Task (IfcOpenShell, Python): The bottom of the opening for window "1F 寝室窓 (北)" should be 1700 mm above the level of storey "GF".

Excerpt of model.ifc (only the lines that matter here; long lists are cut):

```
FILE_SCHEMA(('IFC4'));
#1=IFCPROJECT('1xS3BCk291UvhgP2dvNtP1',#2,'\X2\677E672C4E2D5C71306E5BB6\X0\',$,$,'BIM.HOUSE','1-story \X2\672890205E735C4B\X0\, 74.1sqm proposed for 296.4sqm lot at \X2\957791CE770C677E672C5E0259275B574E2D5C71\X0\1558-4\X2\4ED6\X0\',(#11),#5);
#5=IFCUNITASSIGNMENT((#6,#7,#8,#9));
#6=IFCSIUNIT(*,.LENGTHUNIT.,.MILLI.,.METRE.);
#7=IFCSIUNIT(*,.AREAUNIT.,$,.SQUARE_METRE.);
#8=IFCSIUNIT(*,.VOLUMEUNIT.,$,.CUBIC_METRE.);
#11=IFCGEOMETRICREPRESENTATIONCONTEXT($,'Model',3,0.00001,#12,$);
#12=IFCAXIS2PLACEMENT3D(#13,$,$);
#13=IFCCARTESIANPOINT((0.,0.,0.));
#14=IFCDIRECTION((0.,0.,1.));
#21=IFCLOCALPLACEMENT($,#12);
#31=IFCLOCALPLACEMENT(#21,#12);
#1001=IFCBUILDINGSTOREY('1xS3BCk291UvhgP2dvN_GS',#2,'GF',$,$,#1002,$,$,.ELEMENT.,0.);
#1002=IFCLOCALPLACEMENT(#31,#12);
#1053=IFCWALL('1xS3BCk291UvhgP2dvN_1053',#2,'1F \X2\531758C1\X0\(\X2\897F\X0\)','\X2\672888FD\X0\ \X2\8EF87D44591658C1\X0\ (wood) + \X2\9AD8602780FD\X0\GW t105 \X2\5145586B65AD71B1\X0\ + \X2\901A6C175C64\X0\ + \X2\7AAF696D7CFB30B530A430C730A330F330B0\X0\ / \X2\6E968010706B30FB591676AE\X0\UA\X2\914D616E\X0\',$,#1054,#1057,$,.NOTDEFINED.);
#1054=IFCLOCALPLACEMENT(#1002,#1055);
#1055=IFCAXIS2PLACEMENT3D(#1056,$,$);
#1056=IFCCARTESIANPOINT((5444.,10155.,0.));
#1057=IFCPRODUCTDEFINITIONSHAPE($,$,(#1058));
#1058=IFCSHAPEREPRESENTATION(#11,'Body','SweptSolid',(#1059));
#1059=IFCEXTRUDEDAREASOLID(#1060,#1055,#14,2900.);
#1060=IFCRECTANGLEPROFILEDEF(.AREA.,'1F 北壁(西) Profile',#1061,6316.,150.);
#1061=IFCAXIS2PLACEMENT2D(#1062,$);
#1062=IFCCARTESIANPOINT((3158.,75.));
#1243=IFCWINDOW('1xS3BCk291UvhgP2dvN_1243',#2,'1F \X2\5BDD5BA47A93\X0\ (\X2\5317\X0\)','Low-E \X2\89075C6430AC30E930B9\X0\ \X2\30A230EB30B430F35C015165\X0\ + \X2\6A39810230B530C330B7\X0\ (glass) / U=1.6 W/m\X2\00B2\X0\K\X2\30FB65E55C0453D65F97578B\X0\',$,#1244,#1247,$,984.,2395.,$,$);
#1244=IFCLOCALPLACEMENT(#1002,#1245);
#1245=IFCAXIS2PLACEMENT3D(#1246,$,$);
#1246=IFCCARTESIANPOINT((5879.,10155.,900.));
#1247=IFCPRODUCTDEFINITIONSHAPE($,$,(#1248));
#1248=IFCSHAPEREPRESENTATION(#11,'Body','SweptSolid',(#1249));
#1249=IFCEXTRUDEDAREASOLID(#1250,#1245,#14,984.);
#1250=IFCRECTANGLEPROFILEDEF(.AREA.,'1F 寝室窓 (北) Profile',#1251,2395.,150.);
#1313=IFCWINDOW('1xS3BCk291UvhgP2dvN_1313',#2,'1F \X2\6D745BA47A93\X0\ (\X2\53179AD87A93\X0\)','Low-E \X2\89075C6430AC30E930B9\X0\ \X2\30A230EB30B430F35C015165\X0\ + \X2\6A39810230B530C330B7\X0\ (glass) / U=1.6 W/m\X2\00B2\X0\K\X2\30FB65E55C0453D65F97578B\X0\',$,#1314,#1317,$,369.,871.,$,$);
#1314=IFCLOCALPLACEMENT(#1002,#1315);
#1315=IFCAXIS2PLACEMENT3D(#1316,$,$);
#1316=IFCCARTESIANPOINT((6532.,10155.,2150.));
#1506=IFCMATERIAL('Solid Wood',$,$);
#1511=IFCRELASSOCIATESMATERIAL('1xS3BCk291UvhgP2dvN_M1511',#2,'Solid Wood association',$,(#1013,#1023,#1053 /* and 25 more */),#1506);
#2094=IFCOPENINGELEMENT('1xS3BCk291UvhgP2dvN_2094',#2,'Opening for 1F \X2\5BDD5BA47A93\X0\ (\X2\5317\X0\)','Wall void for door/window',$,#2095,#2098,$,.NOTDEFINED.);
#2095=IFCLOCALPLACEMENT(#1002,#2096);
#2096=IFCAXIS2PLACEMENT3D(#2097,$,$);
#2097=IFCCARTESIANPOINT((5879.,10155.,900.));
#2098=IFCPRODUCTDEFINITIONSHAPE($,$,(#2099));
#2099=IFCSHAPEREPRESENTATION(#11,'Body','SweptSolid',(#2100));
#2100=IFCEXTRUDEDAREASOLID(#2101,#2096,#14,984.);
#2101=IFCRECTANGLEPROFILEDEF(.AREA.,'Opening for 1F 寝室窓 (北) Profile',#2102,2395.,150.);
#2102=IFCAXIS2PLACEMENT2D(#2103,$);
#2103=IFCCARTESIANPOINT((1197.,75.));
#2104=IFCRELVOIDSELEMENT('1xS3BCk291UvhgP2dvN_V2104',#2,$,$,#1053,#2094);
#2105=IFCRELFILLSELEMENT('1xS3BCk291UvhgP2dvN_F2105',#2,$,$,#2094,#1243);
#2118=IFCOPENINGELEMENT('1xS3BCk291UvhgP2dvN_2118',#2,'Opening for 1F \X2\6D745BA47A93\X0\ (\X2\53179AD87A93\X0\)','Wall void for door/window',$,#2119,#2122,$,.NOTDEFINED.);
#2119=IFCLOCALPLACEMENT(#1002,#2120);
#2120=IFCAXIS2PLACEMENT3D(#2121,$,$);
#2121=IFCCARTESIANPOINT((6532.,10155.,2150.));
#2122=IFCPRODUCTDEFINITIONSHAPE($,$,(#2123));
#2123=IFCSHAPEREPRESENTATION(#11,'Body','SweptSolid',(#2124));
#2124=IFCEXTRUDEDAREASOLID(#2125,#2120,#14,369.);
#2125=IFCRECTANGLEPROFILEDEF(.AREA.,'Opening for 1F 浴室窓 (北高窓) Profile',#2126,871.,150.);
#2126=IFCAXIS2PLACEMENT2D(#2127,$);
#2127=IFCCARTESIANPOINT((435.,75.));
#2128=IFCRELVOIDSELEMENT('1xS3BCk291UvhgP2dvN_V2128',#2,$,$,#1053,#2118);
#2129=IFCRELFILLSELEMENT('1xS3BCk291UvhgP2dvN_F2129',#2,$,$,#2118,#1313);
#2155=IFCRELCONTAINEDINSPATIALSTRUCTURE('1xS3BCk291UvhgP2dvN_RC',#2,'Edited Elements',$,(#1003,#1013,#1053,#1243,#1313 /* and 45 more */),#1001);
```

```python
import numpy as np
import ifcopenshell
import ifcopenshell.api.geometry
import ifcopenshell.geom
import ifcopenshell.util.element
import ifcopenshell.util.placement
import ifcopenshell.util.shape
import ifcopenshell.util.unit

model = ifcopenshell.open("model.ifc")
unit_scale = ifcopenshell.util.unit.calculate_unit_scale(model)

window = model.by_guid("1xS3BCk291UvhgP2dvN_1243")
opening = window.FillsVoids[0].RelatingOpeningElement
storey = ifcopenshell.util.element.get_container(window, ifc_class="IfcBuildingStorey")
level = ifcopenshell.util.placement.get_local_placement(storey.ObjectPlacement)[2, 3]

# The opening's origin need not be at the sill, so measure its lowest point.
shape = ifcopenshell.geom.create_shape(ifcopenshell.geom.settings(), opening)
bottom = ifcopenshell.util.shape.get_shape_bottom_elevation(shape, shape.geometry) / unit_scale
dz = level + 1700.0 - bottom

shift = np.array([0.0, 0.0, dz])
# The window is not placed relative to its opening, so move both.
for product in (opening, window):
    matrix = ifcopenshell.util.placement.get_local_placement(product.ObjectPlacement)
    matrix[:3, 3] += shift
    ifcopenshell.api.geometry.edit_object_placement(model, product=product, matrix=matrix, is_si=False)

print(f"moved by {dz * unit_scale:+.3f} m")

model.write("model_v2.ifc")
```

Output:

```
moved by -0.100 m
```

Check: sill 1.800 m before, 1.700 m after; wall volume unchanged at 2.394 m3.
